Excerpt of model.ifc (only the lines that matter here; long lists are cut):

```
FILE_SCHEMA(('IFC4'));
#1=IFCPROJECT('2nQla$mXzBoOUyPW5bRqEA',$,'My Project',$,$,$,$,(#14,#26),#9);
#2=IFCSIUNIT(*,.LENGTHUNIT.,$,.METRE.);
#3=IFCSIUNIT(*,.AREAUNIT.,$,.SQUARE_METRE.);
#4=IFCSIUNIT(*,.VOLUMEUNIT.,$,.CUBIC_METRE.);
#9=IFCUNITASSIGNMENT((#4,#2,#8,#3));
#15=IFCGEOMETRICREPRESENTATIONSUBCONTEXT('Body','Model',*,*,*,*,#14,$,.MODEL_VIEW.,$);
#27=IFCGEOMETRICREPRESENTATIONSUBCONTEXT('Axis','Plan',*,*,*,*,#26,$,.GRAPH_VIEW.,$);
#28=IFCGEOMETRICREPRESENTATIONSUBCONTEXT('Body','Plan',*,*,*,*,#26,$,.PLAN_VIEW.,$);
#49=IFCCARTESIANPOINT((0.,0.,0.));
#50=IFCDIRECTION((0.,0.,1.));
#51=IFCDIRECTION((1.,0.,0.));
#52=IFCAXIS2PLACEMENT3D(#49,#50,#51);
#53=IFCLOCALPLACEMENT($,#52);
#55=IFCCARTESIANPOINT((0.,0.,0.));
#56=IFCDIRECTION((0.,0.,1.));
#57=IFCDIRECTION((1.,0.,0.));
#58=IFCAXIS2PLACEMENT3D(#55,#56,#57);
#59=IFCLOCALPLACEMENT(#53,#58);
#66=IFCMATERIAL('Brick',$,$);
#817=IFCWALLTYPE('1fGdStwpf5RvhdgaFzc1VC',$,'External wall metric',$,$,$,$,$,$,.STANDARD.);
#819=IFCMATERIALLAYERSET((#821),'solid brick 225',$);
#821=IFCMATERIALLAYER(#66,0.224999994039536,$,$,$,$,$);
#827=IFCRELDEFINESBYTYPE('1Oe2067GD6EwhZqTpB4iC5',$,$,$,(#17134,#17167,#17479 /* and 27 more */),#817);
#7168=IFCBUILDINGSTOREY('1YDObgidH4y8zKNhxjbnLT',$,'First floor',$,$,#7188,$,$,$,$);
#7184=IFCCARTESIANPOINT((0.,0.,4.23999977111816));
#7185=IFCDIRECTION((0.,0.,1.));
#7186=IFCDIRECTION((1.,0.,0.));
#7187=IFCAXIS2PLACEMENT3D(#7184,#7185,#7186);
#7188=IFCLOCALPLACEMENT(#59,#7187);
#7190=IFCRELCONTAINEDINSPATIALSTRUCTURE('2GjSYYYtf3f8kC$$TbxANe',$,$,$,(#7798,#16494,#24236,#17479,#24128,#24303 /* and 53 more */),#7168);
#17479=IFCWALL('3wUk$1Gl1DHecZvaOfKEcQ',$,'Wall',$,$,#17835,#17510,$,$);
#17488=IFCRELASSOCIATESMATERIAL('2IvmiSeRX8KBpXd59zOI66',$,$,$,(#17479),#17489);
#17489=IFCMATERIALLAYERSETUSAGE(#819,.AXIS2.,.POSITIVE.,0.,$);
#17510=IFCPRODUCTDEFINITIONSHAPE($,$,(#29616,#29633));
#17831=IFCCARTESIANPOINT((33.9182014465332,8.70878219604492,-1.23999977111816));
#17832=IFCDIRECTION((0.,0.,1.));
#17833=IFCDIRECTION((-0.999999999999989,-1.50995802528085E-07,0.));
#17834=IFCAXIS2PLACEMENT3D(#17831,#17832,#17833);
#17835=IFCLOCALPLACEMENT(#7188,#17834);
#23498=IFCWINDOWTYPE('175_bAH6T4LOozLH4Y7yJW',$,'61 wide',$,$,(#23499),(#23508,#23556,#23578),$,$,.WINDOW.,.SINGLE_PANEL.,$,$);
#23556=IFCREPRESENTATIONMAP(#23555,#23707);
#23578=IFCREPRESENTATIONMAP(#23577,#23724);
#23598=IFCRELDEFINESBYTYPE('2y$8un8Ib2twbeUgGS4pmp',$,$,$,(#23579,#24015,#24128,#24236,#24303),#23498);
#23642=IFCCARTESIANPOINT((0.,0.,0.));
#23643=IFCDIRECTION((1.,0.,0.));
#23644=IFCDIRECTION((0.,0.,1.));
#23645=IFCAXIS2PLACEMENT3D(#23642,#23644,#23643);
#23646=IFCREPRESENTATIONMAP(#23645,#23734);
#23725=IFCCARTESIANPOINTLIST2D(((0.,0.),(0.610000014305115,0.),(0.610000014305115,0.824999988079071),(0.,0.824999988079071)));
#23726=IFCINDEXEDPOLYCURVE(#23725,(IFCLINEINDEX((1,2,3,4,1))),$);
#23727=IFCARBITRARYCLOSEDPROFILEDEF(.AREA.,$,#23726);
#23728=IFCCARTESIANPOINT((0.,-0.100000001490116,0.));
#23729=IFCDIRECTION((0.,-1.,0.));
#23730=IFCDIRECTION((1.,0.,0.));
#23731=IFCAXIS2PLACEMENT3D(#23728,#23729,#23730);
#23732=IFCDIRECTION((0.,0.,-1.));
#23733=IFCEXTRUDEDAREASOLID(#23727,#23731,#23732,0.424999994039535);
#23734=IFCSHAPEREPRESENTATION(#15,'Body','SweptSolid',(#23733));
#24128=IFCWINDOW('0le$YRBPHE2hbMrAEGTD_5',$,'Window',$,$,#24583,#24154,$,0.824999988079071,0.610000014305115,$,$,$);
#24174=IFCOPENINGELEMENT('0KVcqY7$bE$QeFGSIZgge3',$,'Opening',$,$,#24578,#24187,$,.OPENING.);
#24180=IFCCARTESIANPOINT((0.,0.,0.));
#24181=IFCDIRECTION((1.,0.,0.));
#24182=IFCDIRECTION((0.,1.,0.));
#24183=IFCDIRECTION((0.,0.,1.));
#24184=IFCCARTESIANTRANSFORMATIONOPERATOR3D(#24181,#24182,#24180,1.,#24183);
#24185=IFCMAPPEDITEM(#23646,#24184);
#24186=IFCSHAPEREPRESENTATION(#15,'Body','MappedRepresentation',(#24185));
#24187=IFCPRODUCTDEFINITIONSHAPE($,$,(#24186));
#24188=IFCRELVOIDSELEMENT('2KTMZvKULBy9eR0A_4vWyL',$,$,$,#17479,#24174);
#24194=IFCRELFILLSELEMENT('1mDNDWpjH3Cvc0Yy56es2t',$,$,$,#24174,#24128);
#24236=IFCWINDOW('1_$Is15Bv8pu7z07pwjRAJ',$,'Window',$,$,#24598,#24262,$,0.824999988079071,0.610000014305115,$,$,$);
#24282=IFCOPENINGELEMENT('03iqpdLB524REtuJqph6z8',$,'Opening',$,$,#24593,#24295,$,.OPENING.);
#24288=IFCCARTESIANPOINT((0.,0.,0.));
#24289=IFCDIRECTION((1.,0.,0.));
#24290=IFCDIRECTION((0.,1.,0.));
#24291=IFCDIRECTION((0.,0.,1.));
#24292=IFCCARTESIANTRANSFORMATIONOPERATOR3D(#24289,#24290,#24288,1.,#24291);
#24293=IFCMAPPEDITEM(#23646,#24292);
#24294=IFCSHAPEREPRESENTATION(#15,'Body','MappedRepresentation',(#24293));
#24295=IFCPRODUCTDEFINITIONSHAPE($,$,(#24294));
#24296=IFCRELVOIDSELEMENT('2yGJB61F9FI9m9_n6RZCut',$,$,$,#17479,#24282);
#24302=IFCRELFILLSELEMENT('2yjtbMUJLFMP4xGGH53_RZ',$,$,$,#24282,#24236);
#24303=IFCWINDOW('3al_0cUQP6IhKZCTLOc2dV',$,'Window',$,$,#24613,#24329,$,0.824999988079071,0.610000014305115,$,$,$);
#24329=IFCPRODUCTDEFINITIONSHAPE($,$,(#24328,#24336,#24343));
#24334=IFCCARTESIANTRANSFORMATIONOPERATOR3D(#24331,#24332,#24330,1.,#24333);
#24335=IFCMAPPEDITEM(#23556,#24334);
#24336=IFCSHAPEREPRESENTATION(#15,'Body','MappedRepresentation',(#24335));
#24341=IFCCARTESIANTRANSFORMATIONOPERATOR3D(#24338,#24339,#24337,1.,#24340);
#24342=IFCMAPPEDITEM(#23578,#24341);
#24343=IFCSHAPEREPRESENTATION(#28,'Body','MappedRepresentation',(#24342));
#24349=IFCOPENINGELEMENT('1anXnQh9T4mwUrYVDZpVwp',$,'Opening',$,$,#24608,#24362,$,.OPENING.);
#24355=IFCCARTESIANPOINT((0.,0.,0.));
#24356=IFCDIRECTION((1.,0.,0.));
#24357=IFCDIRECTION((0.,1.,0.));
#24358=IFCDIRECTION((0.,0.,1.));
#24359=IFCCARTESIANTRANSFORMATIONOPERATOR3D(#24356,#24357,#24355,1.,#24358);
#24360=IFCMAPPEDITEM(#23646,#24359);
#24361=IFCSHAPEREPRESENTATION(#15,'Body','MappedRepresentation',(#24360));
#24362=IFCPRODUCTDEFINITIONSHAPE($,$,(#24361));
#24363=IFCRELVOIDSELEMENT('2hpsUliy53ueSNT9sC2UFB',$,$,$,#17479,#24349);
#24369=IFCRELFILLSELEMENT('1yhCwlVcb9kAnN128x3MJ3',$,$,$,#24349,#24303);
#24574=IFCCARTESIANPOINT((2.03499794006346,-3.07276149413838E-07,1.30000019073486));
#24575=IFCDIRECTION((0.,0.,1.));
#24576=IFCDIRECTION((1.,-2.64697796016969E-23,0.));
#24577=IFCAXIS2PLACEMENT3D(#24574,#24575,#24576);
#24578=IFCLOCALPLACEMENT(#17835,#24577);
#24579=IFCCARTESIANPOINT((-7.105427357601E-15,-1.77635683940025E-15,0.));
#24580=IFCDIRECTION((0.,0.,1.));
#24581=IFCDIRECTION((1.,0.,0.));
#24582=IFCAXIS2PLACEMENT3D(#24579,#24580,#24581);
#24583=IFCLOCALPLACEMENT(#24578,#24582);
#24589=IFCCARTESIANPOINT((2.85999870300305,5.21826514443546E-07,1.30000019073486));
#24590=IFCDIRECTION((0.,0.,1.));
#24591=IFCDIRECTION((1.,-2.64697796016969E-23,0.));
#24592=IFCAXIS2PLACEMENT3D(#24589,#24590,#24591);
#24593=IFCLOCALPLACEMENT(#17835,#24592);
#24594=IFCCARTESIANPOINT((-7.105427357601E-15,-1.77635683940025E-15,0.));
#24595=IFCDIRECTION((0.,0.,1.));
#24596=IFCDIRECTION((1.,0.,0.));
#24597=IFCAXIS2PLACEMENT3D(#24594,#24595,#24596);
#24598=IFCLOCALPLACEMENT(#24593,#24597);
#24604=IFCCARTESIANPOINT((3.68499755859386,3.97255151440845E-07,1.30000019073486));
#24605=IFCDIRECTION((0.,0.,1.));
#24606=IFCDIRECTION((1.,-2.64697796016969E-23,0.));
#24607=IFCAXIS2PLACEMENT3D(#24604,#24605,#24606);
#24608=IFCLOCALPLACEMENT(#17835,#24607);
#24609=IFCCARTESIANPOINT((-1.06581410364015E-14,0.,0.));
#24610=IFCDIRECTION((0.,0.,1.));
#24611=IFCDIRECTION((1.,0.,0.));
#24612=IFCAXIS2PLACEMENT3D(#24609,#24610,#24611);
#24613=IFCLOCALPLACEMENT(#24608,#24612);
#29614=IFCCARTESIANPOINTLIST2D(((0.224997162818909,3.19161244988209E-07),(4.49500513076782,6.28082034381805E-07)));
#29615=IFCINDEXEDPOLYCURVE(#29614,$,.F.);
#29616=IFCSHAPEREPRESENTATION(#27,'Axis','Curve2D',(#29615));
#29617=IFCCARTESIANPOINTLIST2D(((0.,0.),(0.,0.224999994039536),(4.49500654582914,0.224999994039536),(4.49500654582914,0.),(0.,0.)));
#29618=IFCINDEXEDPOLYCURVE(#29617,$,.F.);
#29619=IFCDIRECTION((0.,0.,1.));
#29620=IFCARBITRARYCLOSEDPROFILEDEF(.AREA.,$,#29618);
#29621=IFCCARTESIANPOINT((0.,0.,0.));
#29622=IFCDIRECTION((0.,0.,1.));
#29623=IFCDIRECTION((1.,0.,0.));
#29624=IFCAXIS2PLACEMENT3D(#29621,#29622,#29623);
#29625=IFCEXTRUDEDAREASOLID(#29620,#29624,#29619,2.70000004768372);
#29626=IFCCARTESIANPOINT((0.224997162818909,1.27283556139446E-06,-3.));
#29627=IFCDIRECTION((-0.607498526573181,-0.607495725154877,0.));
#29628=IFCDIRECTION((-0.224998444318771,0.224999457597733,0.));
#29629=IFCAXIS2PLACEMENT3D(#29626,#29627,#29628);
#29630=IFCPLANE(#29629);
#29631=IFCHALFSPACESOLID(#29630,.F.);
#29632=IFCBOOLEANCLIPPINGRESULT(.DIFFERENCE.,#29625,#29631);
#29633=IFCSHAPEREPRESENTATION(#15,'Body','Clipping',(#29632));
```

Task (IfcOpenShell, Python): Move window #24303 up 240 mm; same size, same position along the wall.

```python
import numpy as np
import ifcopenshell
import ifcopenshell.api.geometry
import ifcopenshell.util.placement
import ifcopenshell.util.unit

model = ifcopenshell.open("model.ifc")
unit_scale = ifcopenshell.util.unit.calculate_unit_scale(model)

window = model.by_guid("3al_0cUQP6IhKZCTLOc2dV")
opening = window.FillsVoids[0].RelatingOpeningElement
dz = 0.24 / unit_scale

shift = np.array([0.0, 0.0, dz])
# The window is placed relative to its opening, so it follows when the opening moves.
matrix = ifcopenshell.util.placement.get_local_placement(opening.ObjectPlacement)
matrix[:3, 3] += shift
ifcopenshell.api.geometry.edit_object_placement(
    model, product=opening, matrix=matrix, is_si=False, should_transform_children=True
)

print(f"moved by {dz * unit_scale:+.3f} m")

model.write("model_updated.ifc")
```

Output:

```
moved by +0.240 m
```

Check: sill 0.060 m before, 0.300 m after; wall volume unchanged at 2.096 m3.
